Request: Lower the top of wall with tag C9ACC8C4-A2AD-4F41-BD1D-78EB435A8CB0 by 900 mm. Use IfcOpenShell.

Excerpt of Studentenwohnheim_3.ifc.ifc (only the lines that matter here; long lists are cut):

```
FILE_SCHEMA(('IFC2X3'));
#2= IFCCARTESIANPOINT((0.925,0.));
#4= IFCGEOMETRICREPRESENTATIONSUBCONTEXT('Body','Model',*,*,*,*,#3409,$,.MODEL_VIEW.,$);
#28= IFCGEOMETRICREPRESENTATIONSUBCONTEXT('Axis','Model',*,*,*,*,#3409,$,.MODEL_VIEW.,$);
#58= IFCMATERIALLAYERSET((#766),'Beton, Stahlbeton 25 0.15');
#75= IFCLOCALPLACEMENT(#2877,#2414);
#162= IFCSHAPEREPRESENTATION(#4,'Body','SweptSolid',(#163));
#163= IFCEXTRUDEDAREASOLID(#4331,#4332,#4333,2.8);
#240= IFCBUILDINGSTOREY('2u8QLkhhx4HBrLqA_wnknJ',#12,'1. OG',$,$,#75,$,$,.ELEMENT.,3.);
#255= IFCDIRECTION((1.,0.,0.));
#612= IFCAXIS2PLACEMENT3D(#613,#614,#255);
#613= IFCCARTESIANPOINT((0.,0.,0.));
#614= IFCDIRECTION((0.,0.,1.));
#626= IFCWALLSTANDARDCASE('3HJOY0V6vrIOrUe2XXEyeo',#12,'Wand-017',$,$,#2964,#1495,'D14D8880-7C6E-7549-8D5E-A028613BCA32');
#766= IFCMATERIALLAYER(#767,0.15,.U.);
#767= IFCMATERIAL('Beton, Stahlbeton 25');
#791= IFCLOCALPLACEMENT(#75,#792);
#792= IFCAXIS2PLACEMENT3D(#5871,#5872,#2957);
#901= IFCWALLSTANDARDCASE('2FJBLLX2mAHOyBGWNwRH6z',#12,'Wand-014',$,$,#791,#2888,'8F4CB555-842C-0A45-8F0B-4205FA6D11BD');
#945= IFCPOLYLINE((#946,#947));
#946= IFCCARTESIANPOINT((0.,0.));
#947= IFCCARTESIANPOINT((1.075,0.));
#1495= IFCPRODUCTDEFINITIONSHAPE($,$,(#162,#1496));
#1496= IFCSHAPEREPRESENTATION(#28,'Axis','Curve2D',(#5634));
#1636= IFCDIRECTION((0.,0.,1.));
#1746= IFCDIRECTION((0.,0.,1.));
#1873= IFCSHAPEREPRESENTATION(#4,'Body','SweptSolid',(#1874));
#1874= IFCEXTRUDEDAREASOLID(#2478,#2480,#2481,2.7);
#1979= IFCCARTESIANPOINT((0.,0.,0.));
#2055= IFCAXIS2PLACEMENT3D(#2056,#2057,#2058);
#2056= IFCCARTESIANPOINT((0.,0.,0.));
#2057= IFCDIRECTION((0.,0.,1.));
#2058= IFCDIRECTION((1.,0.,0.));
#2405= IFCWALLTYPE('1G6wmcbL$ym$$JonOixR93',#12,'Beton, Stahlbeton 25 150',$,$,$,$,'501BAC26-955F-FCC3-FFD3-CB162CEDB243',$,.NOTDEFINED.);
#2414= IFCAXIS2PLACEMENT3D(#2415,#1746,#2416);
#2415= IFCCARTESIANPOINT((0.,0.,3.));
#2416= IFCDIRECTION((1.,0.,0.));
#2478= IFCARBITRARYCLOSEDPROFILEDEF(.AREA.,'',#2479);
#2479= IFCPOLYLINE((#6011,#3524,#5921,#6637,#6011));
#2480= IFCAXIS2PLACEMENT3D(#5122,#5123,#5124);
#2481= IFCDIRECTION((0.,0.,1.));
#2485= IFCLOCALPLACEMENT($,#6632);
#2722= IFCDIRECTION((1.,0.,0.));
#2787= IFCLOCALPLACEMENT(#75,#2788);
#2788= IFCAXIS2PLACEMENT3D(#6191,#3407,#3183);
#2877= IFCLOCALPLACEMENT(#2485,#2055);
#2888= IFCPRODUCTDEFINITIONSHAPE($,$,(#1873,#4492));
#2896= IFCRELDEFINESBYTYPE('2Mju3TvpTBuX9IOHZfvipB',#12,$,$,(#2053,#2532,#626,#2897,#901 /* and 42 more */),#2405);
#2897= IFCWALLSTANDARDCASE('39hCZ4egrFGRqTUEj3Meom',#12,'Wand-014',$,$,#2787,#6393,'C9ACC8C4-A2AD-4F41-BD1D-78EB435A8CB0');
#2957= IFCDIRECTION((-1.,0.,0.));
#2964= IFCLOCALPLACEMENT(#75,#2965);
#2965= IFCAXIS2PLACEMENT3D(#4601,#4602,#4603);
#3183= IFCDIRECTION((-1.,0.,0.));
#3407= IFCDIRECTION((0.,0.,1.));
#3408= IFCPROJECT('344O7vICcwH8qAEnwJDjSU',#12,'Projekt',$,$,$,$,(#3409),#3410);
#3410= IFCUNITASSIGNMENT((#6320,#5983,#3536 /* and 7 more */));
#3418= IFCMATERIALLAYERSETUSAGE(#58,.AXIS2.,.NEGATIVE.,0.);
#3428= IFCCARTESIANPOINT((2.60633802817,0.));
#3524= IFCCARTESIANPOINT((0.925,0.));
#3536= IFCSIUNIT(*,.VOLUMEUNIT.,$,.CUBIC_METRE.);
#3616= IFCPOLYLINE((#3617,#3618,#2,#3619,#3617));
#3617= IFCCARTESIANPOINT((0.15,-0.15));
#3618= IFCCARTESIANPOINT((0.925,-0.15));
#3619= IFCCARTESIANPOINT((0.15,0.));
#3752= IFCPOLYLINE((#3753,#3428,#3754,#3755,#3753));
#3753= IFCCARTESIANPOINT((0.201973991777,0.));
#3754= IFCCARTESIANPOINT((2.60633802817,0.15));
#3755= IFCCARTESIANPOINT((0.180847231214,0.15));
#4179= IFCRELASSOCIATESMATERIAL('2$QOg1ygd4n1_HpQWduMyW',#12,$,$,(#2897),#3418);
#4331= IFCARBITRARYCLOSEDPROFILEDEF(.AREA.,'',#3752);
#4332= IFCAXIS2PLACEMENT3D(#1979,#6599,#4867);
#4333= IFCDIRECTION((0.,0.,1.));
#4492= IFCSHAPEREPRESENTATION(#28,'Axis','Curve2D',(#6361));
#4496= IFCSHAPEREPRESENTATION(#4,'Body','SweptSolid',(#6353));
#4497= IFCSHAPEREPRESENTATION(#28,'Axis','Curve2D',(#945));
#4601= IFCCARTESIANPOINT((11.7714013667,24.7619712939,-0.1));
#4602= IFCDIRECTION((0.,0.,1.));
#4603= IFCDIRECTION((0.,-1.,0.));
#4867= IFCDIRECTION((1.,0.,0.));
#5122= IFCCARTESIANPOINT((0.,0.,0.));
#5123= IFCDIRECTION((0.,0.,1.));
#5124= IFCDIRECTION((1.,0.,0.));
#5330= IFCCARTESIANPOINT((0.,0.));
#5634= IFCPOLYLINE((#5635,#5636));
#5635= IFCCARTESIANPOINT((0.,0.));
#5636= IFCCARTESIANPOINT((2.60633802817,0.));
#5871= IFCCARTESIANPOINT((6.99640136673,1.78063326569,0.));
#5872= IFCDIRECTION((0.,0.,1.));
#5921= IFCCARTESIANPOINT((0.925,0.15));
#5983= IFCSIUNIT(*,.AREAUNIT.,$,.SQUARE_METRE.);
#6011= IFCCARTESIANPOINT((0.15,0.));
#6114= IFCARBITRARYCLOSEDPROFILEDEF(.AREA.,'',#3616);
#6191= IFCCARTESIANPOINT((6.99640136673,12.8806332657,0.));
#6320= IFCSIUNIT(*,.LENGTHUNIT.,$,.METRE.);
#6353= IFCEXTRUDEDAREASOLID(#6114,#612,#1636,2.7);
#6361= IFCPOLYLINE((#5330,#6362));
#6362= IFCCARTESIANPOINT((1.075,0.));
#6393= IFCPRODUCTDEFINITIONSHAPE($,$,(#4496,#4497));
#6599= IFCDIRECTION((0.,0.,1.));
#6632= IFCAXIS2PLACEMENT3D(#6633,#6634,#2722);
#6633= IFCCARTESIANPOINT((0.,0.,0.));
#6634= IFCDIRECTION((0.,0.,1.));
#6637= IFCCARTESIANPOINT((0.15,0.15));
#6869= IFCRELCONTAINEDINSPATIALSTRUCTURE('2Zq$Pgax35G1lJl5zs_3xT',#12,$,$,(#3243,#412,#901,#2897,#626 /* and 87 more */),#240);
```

```python
import ifcopenshell
import ifcopenshell.geom
import ifcopenshell.util.representation
import ifcopenshell.util.shape
import ifcopenshell.util.unit

model = ifcopenshell.open("Studentenwohnheim_3.ifc.ifc")
unit_scale = ifcopenshell.util.unit.calculate_unit_scale(model)
settings = ifcopenshell.geom.settings()


def volume(element):
    """Net volume in cubic metres, openings subtracted."""
    shape = ifcopenshell.geom.create_shape(settings, element)
    return ifcopenshell.util.shape.get_volume(shape.geometry)


wall = model.by_guid("39hCZ4egrFGRqTUEj3Meom")
before = volume(wall)

body = ifcopenshell.util.representation.get_representation(wall, "Model", "Body")
solid = body.Items[0]
old_height = solid.Depth
solid.Depth -= 0.9 / unit_scale
after = volume(wall)

print(f"height {old_height:g} -> {solid.Depth:g}, volume {before:.3f} -> {after:.3f} m3")

model.write("Studentenwohnheim_3.ifc_rev.ifc")
```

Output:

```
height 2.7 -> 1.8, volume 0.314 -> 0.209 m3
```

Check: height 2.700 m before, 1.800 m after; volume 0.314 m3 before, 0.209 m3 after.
